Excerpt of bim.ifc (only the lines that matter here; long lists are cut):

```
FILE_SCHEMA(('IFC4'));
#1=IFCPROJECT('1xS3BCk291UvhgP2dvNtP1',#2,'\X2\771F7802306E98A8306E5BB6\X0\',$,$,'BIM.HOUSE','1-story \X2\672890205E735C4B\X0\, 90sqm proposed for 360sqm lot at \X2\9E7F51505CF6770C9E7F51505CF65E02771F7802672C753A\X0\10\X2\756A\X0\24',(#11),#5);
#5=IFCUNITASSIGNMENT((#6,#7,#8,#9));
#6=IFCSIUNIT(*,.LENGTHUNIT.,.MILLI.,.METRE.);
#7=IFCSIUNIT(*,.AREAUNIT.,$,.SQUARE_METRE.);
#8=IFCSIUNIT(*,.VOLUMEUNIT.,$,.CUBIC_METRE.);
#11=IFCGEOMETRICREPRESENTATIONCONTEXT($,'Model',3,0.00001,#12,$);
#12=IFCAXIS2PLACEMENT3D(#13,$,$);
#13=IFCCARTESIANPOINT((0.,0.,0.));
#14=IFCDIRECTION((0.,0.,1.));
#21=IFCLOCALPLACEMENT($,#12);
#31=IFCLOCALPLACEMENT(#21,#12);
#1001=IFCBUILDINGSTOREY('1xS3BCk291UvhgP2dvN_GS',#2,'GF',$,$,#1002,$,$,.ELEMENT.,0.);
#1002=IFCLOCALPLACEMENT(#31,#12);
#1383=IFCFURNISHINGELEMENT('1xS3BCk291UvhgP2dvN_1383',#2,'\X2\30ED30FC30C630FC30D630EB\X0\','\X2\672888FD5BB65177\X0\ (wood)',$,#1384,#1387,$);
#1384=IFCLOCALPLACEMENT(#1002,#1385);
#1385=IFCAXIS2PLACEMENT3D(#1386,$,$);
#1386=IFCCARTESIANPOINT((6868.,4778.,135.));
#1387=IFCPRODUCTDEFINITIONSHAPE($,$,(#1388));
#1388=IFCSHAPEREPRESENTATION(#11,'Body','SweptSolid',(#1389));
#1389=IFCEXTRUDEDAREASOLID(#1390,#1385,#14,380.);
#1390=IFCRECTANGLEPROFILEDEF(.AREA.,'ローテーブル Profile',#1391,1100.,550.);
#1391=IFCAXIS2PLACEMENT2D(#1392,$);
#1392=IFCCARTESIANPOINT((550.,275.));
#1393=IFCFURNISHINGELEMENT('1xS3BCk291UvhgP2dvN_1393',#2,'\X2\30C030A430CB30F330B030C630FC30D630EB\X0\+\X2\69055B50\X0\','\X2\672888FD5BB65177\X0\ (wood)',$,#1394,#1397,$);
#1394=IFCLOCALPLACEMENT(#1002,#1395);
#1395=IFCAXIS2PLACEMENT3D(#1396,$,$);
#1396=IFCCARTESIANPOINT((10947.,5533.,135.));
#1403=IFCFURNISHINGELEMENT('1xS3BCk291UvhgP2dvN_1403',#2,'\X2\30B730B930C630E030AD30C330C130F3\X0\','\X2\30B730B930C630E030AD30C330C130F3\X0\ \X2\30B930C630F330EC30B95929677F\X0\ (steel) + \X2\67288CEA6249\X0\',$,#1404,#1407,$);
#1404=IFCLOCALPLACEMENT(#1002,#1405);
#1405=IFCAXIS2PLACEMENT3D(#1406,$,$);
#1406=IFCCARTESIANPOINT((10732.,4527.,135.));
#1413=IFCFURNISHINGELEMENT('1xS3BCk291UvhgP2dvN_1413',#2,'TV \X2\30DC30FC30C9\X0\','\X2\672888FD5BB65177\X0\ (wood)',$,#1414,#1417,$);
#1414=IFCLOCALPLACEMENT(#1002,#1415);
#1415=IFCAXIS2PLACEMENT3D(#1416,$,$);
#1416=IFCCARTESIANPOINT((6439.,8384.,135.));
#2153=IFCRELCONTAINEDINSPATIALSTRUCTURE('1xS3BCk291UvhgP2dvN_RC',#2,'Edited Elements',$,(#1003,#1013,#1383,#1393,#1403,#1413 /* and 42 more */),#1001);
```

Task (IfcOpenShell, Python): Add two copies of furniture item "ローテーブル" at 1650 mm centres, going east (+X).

```python
import numpy as np
import ifcopenshell
import ifcopenshell.api.geometry
import ifcopenshell.api.root
import ifcopenshell.util.element
import ifcopenshell.util.placement
import ifcopenshell.util.unit

model = ifcopenshell.open("bim.ifc")
unit_scale = ifcopenshell.util.unit.calculate_unit_scale(model)


def reuse_history(source, copy):
    """copy_class also copies each property set's owner history, people and application; keep the originals."""
    for rel in copy.IsDefinedBy:
        if rel.is_a("IfcRelDefinesByProperties") and (history := rel.RelatingPropertyDefinition.OwnerHistory):
            rel.RelatingPropertyDefinition.OwnerHistory = source.OwnerHistory
            ifcopenshell.util.element.remove_deep2(model, history)


source = model.by_id(1383)
base = ifcopenshell.util.placement.get_local_placement(source.ObjectPlacement)
step = np.array([1.0, 0.0, 0.0]) * 1.65 / unit_scale

for i in range(1, 3):
    copy = ifcopenshell.api.root.copy_class(model, product=source)
    copy.Representation = ifcopenshell.util.element.copy_deep(
        model, source.Representation, exclude=["IfcGeometricRepresentationContext", "IfcRepresentationMap"]
    )
    reuse_history(source, copy)
    matrix = base.copy()
    matrix[:3, 3] += i * step
    print("added at", matrix[:3, 3].round(3) + 0.0)
    ifcopenshell.api.geometry.edit_object_placement(model, product=copy, matrix=matrix, is_si=False)

model.write("bim_updated.ifc")
```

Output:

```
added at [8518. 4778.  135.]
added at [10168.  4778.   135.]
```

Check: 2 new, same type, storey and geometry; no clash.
